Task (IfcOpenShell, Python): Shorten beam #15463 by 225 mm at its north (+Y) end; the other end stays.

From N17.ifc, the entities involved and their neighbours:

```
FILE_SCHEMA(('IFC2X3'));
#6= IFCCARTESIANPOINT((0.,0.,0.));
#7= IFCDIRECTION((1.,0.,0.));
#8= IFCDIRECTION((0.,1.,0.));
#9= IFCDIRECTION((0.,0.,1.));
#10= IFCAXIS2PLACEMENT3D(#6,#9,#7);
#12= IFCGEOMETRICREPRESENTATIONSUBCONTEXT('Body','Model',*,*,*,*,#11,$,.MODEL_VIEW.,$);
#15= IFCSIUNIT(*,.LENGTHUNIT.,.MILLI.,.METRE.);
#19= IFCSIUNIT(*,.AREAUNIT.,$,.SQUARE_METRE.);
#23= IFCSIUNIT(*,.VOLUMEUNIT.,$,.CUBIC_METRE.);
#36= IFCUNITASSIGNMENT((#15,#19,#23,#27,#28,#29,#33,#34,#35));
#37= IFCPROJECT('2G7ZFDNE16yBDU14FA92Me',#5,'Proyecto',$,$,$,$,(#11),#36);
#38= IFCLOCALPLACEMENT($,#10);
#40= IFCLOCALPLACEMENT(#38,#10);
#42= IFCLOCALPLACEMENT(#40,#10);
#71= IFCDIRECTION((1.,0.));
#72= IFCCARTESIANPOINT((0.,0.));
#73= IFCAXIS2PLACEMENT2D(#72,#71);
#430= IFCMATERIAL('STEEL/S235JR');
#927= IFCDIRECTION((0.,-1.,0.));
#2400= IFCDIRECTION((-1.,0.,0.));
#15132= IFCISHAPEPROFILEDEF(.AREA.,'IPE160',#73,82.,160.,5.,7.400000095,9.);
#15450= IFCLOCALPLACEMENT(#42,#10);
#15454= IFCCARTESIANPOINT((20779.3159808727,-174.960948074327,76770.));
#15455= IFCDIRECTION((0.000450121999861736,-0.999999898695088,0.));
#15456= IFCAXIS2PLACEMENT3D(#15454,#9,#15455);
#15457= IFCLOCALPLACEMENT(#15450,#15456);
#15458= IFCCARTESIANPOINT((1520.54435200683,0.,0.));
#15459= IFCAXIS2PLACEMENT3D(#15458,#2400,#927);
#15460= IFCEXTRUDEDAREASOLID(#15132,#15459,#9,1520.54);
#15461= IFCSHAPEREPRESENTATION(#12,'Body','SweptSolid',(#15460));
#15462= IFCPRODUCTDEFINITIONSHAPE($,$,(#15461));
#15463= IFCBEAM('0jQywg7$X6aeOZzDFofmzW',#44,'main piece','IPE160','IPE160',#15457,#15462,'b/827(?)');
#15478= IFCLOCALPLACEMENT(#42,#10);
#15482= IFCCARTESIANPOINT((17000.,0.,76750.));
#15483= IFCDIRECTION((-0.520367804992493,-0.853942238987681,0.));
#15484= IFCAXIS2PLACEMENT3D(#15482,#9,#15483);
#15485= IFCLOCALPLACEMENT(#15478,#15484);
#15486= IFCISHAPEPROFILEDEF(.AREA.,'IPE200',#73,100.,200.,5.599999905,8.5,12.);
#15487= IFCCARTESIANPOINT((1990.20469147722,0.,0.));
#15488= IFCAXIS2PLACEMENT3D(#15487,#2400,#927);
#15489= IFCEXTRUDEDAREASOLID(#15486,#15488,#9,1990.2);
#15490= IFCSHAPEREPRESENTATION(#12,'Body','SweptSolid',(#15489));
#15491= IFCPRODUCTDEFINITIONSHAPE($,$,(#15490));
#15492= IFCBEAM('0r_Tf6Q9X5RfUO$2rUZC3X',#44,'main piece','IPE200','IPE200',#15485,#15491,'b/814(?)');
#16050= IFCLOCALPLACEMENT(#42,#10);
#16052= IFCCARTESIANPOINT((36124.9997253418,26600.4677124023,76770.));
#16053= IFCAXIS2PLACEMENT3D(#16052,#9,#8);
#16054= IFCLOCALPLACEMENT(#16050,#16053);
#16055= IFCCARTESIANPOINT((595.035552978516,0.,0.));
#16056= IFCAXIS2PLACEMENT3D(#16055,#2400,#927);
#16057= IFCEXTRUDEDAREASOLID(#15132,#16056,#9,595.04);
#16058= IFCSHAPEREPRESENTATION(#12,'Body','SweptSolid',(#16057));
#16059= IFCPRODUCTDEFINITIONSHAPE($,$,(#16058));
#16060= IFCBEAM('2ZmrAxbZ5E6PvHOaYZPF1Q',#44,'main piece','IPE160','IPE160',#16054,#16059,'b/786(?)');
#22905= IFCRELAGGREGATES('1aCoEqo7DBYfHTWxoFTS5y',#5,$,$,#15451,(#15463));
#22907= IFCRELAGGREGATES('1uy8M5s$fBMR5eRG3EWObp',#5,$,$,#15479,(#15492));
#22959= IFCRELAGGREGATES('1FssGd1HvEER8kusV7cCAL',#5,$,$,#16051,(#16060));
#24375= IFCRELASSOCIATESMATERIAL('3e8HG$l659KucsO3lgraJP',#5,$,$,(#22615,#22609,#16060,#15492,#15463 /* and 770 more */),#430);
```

```python
import ifcopenshell
import ifcopenshell.util.representation

model = ifcopenshell.open("N17.ifc")

member = model.by_id(15463)
change = -225.0

# The extrusion runs towards the end named, so only its depth changes.
body = ifcopenshell.util.representation.get_representation(member, "Model", "Body")
solid = body.Items[0]
old_length = solid.Depth
solid.Depth += change

print(f"length {old_length:g} -> {solid.Depth:g}")

model.write("N17_v2.ifc")
```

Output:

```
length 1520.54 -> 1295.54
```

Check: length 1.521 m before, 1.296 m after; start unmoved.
